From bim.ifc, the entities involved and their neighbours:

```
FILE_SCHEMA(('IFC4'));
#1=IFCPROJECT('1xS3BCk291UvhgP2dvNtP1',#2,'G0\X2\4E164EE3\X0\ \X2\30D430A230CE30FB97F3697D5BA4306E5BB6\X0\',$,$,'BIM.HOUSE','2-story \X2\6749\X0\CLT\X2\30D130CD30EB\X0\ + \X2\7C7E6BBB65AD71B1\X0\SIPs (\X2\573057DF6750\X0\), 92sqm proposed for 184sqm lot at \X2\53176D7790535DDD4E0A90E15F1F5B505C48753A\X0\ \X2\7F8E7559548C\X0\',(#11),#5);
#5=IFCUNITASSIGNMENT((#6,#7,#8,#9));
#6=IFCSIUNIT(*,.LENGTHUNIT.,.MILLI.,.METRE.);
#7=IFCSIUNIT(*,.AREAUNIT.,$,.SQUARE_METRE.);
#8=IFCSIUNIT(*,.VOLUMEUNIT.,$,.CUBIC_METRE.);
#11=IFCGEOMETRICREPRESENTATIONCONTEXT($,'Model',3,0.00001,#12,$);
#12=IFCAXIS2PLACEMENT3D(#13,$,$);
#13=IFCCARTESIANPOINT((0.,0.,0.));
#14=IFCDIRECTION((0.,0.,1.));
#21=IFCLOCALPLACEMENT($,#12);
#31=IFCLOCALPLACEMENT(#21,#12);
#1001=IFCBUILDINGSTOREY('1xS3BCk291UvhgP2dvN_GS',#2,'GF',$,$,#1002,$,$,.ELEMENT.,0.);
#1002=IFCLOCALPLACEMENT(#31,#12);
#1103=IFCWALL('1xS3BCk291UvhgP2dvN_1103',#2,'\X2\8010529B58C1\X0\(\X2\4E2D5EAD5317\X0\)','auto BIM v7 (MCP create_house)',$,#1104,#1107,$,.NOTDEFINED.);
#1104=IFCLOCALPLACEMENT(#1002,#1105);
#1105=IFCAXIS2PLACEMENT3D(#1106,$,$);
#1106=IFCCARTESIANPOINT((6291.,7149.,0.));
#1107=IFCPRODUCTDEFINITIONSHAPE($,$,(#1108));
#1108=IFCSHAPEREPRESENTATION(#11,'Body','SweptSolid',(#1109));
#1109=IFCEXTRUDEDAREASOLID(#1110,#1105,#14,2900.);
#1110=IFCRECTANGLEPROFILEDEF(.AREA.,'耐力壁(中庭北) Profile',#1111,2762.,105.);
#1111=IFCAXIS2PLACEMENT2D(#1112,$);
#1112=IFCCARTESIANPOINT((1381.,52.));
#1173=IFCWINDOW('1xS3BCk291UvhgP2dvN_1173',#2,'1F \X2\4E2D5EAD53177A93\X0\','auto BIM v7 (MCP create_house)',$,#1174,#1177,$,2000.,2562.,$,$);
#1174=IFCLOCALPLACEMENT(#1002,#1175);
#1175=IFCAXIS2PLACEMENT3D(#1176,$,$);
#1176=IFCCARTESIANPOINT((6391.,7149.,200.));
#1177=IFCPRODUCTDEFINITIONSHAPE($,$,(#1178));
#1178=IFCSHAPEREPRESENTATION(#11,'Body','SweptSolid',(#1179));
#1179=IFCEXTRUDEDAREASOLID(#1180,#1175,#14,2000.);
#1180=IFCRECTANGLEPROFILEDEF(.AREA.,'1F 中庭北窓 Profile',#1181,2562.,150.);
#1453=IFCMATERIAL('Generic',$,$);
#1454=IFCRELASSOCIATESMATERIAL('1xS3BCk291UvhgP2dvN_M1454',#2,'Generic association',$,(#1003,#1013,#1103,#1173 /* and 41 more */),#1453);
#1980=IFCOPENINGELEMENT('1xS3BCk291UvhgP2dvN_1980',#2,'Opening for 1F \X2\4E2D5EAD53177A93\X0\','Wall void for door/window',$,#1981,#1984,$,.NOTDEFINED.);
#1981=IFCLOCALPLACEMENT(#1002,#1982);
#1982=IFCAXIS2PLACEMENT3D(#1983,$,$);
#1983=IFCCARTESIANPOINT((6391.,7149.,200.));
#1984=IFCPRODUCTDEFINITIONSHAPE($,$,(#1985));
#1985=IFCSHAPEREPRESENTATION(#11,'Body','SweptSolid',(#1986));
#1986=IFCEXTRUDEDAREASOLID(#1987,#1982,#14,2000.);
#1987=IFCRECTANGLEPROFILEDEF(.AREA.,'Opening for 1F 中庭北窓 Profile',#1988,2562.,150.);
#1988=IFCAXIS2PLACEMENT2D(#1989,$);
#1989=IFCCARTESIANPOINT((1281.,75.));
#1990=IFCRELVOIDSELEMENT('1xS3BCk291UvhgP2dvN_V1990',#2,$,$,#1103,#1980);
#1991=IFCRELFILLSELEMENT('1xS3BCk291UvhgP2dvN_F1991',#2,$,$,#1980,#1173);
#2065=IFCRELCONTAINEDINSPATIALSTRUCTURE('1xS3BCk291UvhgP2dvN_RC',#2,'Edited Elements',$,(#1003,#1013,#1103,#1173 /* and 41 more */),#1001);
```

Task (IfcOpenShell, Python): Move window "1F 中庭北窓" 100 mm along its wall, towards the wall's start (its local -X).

```python
import ifcopenshell
import ifcopenshell.api.geometry
import ifcopenshell.util.placement

model = ifcopenshell.open("bim.ifc")

window = model.by_id(1173)
opening = window.FillsVoids[0].RelatingOpeningElement
wall = opening.VoidsElements[0].RelatingBuildingElement

wall_matrix = ifcopenshell.util.placement.get_local_placement(wall.ObjectPlacement)
shift = wall_matrix[:3, 0] * -100.0
before = ifcopenshell.util.placement.get_local_placement(window.ObjectPlacement)[:3, 3].copy()

# The window is not placed relative to its opening, so move both.
for product in (opening, window):
    matrix = ifcopenshell.util.placement.get_local_placement(product.ObjectPlacement)
    matrix[:3, 3] += shift
    ifcopenshell.api.geometry.edit_object_placement(model, product=product, matrix=matrix, is_si=False)

after = ifcopenshell.util.placement.get_local_placement(window.ObjectPlacement)[:3, 3]
print("window moved by", (after - before).round(3) + 0.0)

model.write("bim_rev.ifc")
```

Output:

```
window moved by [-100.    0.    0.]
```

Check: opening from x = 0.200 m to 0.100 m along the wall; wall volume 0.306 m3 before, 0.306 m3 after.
